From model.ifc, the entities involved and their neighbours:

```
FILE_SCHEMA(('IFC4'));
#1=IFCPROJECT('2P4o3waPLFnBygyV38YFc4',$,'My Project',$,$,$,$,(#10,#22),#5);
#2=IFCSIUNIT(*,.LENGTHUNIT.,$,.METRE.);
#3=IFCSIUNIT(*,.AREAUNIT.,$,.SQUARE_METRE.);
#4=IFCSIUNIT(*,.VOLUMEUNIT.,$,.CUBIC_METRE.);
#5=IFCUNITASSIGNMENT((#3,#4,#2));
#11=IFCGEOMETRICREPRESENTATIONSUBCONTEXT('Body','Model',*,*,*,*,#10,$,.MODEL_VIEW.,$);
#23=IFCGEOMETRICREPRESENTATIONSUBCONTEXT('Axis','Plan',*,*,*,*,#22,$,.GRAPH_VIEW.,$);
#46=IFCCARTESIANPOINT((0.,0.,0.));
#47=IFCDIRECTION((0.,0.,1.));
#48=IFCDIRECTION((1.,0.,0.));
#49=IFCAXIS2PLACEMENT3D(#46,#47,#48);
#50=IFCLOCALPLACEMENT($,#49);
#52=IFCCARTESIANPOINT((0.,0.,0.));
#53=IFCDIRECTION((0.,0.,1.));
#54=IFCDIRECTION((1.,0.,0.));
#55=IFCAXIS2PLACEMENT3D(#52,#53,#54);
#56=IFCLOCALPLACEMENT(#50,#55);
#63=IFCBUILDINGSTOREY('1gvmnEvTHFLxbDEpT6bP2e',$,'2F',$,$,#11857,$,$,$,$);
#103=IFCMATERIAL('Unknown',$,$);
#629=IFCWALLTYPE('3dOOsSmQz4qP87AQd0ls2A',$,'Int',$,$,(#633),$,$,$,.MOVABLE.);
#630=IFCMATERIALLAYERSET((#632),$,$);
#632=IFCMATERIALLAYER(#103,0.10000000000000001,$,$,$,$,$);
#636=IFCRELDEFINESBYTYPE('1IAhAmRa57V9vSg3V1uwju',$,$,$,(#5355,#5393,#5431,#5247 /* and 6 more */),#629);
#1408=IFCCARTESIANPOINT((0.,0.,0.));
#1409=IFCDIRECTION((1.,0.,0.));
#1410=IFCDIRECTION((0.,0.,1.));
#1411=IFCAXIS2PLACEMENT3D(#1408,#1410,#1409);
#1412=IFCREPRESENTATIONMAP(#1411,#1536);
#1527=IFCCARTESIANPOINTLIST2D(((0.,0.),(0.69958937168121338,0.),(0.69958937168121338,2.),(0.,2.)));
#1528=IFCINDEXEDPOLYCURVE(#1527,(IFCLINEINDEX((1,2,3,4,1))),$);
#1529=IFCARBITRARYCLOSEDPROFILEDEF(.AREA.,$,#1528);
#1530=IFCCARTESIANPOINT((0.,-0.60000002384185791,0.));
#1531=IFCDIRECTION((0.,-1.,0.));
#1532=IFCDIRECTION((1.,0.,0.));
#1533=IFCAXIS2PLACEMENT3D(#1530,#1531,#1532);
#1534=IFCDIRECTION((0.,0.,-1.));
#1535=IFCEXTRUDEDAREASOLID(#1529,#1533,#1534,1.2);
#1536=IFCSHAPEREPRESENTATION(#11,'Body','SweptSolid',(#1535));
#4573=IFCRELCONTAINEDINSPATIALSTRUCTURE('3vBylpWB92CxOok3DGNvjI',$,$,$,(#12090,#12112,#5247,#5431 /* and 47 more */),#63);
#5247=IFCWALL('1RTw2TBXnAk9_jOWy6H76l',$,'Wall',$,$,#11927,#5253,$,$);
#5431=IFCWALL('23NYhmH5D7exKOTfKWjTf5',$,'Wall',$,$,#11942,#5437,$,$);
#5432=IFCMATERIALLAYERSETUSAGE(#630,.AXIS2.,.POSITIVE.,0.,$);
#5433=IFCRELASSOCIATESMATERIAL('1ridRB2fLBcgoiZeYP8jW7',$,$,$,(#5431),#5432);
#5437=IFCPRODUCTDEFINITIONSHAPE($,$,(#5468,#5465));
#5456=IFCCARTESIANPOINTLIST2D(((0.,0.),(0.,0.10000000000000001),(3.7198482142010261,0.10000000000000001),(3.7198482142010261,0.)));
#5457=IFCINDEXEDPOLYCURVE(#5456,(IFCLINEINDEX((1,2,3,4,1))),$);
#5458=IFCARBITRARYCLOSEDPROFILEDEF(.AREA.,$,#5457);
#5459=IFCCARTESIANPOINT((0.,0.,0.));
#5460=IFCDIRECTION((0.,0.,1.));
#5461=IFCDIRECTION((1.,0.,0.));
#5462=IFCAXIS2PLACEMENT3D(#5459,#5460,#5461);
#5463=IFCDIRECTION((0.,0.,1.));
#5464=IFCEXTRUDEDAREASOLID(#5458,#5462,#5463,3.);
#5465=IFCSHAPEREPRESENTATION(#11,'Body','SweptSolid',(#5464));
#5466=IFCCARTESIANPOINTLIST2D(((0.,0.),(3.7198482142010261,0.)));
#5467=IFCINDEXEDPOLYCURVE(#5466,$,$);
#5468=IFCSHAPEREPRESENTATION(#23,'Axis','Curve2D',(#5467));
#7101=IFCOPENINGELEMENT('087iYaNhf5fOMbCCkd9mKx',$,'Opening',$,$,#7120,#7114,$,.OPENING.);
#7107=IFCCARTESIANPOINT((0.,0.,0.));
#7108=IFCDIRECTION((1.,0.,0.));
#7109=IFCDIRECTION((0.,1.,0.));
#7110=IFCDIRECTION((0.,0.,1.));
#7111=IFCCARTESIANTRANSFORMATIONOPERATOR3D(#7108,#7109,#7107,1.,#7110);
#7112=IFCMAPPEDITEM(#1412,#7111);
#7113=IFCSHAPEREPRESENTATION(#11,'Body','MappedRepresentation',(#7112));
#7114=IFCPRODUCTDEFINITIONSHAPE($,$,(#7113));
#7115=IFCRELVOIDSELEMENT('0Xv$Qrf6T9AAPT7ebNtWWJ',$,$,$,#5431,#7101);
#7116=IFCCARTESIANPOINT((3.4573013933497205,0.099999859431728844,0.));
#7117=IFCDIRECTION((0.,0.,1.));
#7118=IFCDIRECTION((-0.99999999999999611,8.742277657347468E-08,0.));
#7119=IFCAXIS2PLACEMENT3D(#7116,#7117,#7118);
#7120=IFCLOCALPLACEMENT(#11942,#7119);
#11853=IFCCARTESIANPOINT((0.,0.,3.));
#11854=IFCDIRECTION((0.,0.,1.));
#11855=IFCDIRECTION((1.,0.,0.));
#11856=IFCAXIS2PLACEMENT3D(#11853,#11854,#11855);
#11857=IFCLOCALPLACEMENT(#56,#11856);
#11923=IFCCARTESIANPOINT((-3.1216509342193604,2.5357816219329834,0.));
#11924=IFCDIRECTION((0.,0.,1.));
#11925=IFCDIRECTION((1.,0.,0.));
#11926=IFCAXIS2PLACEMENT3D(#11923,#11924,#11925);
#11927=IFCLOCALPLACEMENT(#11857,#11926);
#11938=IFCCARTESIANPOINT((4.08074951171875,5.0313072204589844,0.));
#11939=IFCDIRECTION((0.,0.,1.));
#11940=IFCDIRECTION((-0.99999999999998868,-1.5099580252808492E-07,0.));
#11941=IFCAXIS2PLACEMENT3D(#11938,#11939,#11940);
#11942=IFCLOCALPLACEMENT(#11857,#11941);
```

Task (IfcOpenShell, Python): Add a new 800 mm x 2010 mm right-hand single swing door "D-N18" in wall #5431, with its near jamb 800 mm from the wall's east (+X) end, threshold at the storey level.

```python
import numpy as np
import ifcopenshell
import ifcopenshell.api.feature
import ifcopenshell.api.geometry
import ifcopenshell.api.root
import ifcopenshell.api.spatial
import ifcopenshell.geom
import ifcopenshell.util.element
import ifcopenshell.util.placement
import ifcopenshell.util.representation
import ifcopenshell.util.shape
import ifcopenshell.util.unit

model = ifcopenshell.open("model.ifc")
unit_scale = ifcopenshell.util.unit.calculate_unit_scale(model)
settings = ifcopenshell.geom.settings()


def volume(element):
    """Net volume in cubic metres, openings subtracted."""
    shape = ifcopenshell.geom.create_shape(settings, element)
    return ifcopenshell.util.shape.get_volume(shape.geometry)


wall = model.by_guid("23NYhmH5D7exKOTfKWjTf5")
storey = ifcopenshell.util.element.get_container(wall, ifc_class="IfcBuildingStorey")
context = ifcopenshell.util.representation.get_context(model, "Model", "Body", "MODEL_VIEW")
before = volume(wall)

width, height, from_end, sill = 0.8, 2.01, 0.8, 0.0  # metres

# The wall runs along its own X axis, and the end named is its -X end.
wall_shape = ifcopenshell.geom.create_shape(settings, wall)
x, y, z = ifcopenshell.util.shape.get_vertices(wall_shape.geometry).T
start = x.min() + from_end
face, thickness = float(y.min()), float(y.max() - y.min())
wall_matrix = ifcopenshell.util.placement.get_local_placement(wall.ObjectPlacement)
level = ifcopenshell.util.placement.get_local_placement(storey.ObjectPlacement)[2, 3]


def in_wall(x, y):
    """Placement at x, y metres in the wall's axes, at sill height."""
    matrix = wall_matrix.copy()
    matrix[:, 3] = wall_matrix @ np.array([x / unit_scale, y / unit_scale, 0.0, 1.0])
    matrix[2, 3] = level + sill / unit_scale
    return matrix


# Opening: a box that overshoots both wall faces by 50 mm.
opening = ifcopenshell.api.root.create_entity(model, ifc_class="IfcOpeningElement", predefined_type="OPENING")
box = ifcopenshell.api.geometry.add_wall_representation(
    model, context=context, length=width, height=height, thickness=thickness + 0.1
)
ifcopenshell.api.geometry.assign_representation(model, product=opening, representation=box)
ifcopenshell.api.geometry.edit_object_placement(model, product=opening, matrix=in_wall(start, face - 0.05), is_si=False)
ifcopenshell.api.feature.add_feature(model, feature=opening, element=wall)

door = ifcopenshell.api.root.create_entity(model, ifc_class="IfcDoor", name="D-N18", predefined_type="DOOR")
door.OverallWidth, door.OverallHeight = width / unit_scale, height / unit_scale
door.OperationType = "SINGLE_SWING_RIGHT"
body = ifcopenshell.api.geometry.add_door_representation(
    model,
    context=context,
    overall_width=door.OverallWidth,
    overall_height=door.OverallHeight,
    operation_type="SINGLE_SWING_RIGHT",
    lining_properties={"LiningDepth": thickness / unit_scale, "ThresholdDepth": thickness / unit_scale},
)
ifcopenshell.api.geometry.assign_representation(model, product=door, representation=body)
ifcopenshell.api.spatial.assign_container(model, products=[door], relating_structure=storey)
ifcopenshell.api.feature.add_filling(model, opening=opening, element=door)

# The lining spans the wall, so the door starts at the wall face.
ifcopenshell.api.geometry.edit_object_placement(model, product=door, matrix=in_wall(start, face), is_si=False)

after = volume(wall)

print(f"wall volume {before:.3f} -> {after:.3f} m3")

model.write("model_edited.ifc")
```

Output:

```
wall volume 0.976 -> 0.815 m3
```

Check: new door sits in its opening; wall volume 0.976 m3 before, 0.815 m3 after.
